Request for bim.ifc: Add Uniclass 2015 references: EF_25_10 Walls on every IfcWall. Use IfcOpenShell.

First a look at what the model holds.

```python
import ifcopenshell

model = ifcopenshell.open("bim.ifc")
print(model.schema)
print("classifications:", [c.Name for c in model.by_type("IfcClassification")])
for ifc_class in ("IfcDoor", "IfcRoof", "IfcStair", "IfcWall", "IfcWindow"):
    print(ifc_class, len(model.by_type(ifc_class)))
```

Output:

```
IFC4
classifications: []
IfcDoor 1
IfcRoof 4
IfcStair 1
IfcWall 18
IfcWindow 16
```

```python
import ifcopenshell
import ifcopenshell.api.classification

model = ifcopenshell.open("bim.ifc")

system = ifcopenshell.api.classification.add_classification(model, classification="Uniclass 2015")

codes = {
    "IfcWall": ("EF_25_10", "Walls"),
}
for ifc_class, (code, name) in codes.items():
    products = model.by_type(ifc_class)
    ifcopenshell.api.classification.add_reference(
        model, products=products, classification=system, identification=code, name=name
    )
    print(code, len(products))

model.write("bim_v2.ifc")
```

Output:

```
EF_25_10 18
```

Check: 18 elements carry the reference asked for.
